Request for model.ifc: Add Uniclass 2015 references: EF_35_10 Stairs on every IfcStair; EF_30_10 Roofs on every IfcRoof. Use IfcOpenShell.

First a look at what the model holds.

```python
import ifcopenshell

model = ifcopenshell.open("model.ifc")
print(model.schema)
print("classifications:", [c.Name for c in model.by_type("IfcClassification")])
for ifc_class in ("IfcDoor", "IfcRoof", "IfcStair", "IfcWall", "IfcWindow"):
    print(ifc_class, len(model.by_type(ifc_class)))
```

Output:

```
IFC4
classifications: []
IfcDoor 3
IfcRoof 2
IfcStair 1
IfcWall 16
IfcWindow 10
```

```python
import ifcopenshell
import ifcopenshell.api.classification

model = ifcopenshell.open("model.ifc")

system = ifcopenshell.api.classification.add_classification(model, classification="Uniclass 2015")

codes = {
    "IfcStair": ("EF_35_10", "Stairs"),
    "IfcRoof": ("EF_30_10", "Roofs"),
}
for ifc_class, (code, name) in codes.items():
    products = model.by_type(ifc_class)
    ifcopenshell.api.classification.add_reference(
        model, products=products, classification=system, identification=code, name=name
    )
    print(code, len(products))

model.write("model-out.ifc")
```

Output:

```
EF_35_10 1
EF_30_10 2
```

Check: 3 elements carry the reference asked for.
